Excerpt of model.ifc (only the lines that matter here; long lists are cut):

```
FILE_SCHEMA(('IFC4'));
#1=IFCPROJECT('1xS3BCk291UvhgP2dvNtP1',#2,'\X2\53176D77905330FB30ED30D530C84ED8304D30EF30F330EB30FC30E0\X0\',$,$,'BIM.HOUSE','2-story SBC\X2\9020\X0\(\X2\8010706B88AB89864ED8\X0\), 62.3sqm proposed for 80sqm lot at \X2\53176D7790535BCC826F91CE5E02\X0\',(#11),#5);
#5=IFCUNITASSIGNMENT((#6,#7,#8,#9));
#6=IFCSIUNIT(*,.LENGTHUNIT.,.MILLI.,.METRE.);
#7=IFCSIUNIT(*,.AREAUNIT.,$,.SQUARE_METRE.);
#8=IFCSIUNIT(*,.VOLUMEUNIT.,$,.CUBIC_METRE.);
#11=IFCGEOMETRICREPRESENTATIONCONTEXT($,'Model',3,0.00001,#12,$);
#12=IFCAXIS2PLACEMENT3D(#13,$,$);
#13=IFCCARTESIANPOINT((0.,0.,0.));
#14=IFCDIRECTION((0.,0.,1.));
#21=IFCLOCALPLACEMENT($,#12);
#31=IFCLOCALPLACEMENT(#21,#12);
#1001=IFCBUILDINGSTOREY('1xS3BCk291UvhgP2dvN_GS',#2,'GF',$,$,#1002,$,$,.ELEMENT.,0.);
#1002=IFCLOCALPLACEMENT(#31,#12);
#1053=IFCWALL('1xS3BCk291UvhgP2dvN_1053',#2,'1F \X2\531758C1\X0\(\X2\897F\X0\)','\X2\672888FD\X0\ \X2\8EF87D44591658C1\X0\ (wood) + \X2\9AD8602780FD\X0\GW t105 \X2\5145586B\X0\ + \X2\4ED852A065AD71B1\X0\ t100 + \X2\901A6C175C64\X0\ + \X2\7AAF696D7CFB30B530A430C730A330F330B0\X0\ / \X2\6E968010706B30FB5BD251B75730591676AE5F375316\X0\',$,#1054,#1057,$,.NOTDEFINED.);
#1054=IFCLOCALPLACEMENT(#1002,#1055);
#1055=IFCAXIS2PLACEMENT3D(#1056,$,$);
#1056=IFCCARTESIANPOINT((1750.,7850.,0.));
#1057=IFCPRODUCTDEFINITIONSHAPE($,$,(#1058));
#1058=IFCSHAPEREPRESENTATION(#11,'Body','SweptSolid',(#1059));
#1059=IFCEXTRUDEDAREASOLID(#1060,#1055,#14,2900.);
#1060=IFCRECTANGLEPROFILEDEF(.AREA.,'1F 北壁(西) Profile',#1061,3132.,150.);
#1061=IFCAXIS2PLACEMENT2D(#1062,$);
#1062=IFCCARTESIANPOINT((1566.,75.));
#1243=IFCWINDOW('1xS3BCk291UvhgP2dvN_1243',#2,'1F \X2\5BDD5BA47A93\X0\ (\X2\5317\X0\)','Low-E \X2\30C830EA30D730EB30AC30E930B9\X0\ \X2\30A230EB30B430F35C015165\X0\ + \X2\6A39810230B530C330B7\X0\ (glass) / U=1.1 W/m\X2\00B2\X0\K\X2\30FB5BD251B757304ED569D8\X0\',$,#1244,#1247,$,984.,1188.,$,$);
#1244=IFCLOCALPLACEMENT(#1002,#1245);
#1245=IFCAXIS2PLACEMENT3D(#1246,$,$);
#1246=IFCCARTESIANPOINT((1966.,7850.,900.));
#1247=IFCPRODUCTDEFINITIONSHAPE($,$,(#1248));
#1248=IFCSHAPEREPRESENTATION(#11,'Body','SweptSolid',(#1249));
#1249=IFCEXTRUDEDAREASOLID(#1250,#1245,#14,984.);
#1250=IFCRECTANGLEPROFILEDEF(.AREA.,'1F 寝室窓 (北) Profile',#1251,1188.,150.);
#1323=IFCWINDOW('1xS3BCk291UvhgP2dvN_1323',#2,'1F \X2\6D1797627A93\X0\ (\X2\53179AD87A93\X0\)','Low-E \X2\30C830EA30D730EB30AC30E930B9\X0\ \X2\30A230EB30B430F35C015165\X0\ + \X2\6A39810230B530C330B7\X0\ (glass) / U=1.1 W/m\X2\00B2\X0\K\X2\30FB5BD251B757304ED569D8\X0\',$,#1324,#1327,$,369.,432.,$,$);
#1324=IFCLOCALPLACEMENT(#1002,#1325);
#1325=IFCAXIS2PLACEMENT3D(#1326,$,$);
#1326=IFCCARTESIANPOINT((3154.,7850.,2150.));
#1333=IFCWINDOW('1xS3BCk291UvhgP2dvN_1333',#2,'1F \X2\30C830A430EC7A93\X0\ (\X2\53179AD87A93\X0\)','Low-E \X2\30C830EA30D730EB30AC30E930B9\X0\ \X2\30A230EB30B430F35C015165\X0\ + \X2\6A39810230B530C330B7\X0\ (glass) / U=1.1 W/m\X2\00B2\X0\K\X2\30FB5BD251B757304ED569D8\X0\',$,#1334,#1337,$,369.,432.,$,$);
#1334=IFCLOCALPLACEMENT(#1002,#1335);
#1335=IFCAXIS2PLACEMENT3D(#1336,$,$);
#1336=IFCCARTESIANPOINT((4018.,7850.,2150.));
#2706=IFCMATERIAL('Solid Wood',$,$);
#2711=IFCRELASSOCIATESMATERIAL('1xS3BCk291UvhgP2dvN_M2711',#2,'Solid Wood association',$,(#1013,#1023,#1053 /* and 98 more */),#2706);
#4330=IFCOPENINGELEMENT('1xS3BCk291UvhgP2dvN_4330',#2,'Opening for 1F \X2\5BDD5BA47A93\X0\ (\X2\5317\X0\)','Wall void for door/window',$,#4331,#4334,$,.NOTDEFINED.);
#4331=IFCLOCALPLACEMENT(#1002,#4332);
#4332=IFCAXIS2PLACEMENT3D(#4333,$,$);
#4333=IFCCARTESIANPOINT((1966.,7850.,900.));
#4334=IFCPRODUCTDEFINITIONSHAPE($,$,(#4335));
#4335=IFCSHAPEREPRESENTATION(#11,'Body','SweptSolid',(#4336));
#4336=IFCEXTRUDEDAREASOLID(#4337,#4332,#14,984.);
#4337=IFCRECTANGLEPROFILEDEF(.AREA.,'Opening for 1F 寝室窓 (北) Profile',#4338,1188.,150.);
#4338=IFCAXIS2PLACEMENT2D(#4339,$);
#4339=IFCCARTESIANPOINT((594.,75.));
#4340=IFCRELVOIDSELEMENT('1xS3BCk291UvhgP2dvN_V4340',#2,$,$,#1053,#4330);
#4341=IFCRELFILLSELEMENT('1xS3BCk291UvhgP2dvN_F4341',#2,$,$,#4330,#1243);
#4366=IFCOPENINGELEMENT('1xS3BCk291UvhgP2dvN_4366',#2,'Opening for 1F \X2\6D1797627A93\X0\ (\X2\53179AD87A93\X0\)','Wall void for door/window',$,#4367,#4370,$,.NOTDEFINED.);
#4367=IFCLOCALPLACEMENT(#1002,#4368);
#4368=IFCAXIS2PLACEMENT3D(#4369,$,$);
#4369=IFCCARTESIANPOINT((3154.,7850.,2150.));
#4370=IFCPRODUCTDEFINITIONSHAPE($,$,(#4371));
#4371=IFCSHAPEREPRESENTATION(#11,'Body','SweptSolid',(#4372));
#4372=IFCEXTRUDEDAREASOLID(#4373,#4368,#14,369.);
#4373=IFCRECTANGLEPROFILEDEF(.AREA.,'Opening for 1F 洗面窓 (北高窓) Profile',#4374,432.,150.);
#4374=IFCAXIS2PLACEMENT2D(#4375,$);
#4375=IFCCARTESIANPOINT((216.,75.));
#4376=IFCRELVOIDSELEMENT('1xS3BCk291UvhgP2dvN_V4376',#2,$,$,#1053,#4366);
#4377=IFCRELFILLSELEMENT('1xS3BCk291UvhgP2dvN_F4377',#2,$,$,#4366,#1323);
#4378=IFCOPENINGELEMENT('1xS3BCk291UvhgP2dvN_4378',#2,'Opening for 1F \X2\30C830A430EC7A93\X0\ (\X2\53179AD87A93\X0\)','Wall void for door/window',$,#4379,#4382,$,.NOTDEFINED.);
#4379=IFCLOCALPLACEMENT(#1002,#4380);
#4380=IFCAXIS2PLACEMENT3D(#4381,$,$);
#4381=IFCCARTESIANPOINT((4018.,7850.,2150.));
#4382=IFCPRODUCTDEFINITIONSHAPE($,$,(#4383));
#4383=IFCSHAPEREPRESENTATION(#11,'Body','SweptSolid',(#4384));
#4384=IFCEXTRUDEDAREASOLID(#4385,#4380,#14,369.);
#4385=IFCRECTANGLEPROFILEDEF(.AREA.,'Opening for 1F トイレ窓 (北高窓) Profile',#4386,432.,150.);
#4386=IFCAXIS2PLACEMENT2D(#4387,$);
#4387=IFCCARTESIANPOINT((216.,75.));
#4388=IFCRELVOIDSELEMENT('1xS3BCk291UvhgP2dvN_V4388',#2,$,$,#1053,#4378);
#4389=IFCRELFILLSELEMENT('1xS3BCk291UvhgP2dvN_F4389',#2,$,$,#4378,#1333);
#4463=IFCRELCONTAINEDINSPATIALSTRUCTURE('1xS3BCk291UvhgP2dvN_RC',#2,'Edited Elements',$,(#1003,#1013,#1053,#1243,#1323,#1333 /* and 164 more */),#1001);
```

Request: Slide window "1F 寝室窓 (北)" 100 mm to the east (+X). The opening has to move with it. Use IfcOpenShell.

```python
import ifcopenshell
import ifcopenshell.api.geometry
import ifcopenshell.util.placement

model = ifcopenshell.open("model.ifc")

window = model.by_id(1243)
opening = window.FillsVoids[0].RelatingOpeningElement
wall = opening.VoidsElements[0].RelatingBuildingElement

wall_matrix = ifcopenshell.util.placement.get_local_placement(wall.ObjectPlacement)
shift = wall_matrix[:3, 0] * 100.0
before = ifcopenshell.util.placement.get_local_placement(window.ObjectPlacement)[:3, 3].copy()

# The window is not placed relative to its opening, so move both.
for product in (opening, window):
    matrix = ifcopenshell.util.placement.get_local_placement(product.ObjectPlacement)
    matrix[:3, 3] += shift
    ifcopenshell.api.geometry.edit_object_placement(model, product=product, matrix=matrix, is_si=False)

after = ifcopenshell.util.placement.get_local_placement(window.ObjectPlacement)[:3, 3]
print("window moved by", (after - before).round(3) + 0.0)

model.write("model-out.ifc")
```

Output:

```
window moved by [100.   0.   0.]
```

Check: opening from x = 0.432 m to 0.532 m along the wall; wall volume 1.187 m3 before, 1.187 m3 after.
